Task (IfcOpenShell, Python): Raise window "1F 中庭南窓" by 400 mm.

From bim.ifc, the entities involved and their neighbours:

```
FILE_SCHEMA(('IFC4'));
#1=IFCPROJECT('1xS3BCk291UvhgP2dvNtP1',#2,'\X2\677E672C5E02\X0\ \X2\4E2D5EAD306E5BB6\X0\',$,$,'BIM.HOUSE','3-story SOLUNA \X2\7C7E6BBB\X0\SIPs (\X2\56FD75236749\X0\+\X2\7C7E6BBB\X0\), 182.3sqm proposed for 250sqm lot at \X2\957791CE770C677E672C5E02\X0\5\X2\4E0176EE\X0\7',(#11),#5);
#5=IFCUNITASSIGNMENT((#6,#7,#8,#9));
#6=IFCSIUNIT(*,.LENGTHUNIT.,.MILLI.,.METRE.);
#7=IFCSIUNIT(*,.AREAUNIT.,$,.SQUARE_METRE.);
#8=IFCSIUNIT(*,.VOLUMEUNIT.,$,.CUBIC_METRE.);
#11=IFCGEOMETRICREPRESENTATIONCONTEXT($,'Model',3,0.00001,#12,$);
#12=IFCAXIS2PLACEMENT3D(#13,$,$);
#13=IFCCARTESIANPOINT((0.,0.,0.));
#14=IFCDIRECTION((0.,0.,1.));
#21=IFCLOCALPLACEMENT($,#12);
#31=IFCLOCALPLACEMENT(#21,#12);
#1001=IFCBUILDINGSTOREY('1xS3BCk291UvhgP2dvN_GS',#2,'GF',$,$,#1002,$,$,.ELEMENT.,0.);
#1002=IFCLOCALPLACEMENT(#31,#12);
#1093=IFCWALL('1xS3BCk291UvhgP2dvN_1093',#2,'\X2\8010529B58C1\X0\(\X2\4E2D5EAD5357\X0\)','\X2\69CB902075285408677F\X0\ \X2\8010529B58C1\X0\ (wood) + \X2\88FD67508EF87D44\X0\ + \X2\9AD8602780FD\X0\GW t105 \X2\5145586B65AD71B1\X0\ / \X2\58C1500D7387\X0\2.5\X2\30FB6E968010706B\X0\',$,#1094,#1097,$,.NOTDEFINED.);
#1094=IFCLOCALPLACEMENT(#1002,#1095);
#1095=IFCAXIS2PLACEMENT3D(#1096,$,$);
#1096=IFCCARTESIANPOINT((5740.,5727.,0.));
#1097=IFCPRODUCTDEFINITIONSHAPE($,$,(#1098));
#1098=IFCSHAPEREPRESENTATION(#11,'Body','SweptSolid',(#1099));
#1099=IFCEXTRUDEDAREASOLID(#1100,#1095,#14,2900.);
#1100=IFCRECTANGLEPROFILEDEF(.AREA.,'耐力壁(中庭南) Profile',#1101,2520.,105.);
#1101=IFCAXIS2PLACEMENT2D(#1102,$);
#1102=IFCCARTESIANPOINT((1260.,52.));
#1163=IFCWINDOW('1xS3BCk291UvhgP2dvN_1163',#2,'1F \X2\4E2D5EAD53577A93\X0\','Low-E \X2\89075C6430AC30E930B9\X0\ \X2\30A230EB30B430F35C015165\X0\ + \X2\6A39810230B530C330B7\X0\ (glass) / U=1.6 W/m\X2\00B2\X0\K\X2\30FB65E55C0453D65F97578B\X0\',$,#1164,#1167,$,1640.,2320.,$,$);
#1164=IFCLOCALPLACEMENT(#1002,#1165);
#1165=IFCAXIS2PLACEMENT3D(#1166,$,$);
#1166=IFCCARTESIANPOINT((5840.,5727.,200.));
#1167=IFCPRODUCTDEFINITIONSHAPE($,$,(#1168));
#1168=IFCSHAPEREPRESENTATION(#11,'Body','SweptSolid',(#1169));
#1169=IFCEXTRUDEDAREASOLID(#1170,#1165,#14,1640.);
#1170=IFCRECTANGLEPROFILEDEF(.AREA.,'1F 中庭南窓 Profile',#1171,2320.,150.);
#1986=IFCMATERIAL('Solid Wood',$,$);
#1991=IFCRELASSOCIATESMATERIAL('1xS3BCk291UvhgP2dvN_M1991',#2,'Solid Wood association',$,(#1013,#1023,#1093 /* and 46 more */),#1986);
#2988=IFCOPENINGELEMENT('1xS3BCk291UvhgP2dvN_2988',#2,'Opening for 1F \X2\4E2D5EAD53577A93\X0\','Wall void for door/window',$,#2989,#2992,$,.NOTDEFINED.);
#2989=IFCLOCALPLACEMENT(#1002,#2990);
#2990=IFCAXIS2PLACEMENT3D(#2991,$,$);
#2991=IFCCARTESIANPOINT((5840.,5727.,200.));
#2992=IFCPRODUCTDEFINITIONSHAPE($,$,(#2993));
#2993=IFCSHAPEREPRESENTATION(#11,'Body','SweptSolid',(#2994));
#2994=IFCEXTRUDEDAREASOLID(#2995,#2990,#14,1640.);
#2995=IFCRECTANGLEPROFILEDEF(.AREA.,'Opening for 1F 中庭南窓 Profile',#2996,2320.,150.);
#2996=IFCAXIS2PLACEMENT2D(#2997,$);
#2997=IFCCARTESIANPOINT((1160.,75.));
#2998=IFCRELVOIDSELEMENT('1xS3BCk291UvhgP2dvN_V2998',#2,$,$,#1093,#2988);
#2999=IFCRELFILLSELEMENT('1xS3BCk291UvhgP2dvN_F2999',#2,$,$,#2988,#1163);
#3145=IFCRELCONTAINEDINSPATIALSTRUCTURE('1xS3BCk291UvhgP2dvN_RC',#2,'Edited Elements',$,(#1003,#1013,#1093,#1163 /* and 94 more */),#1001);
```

```python
import numpy as np
import ifcopenshell
import ifcopenshell.api.geometry
import ifcopenshell.util.placement
import ifcopenshell.util.unit

model = ifcopenshell.open("bim.ifc")
unit_scale = ifcopenshell.util.unit.calculate_unit_scale(model)

window = model.by_guid("1xS3BCk291UvhgP2dvN_1163")
opening = window.FillsVoids[0].RelatingOpeningElement
dz = 400.0

shift = np.array([0.0, 0.0, dz])
# The window is not placed relative to its opening, so move both.
for product in (opening, window):
    matrix = ifcopenshell.util.placement.get_local_placement(product.ObjectPlacement)
    matrix[:3, 3] += shift
    ifcopenshell.api.geometry.edit_object_placement(model, product=product, matrix=matrix, is_si=False)

print(f"moved by {dz * unit_scale:+.3f} m")

model.write("bim_rev.ifc")
```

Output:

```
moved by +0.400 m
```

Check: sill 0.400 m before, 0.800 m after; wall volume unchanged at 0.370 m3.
